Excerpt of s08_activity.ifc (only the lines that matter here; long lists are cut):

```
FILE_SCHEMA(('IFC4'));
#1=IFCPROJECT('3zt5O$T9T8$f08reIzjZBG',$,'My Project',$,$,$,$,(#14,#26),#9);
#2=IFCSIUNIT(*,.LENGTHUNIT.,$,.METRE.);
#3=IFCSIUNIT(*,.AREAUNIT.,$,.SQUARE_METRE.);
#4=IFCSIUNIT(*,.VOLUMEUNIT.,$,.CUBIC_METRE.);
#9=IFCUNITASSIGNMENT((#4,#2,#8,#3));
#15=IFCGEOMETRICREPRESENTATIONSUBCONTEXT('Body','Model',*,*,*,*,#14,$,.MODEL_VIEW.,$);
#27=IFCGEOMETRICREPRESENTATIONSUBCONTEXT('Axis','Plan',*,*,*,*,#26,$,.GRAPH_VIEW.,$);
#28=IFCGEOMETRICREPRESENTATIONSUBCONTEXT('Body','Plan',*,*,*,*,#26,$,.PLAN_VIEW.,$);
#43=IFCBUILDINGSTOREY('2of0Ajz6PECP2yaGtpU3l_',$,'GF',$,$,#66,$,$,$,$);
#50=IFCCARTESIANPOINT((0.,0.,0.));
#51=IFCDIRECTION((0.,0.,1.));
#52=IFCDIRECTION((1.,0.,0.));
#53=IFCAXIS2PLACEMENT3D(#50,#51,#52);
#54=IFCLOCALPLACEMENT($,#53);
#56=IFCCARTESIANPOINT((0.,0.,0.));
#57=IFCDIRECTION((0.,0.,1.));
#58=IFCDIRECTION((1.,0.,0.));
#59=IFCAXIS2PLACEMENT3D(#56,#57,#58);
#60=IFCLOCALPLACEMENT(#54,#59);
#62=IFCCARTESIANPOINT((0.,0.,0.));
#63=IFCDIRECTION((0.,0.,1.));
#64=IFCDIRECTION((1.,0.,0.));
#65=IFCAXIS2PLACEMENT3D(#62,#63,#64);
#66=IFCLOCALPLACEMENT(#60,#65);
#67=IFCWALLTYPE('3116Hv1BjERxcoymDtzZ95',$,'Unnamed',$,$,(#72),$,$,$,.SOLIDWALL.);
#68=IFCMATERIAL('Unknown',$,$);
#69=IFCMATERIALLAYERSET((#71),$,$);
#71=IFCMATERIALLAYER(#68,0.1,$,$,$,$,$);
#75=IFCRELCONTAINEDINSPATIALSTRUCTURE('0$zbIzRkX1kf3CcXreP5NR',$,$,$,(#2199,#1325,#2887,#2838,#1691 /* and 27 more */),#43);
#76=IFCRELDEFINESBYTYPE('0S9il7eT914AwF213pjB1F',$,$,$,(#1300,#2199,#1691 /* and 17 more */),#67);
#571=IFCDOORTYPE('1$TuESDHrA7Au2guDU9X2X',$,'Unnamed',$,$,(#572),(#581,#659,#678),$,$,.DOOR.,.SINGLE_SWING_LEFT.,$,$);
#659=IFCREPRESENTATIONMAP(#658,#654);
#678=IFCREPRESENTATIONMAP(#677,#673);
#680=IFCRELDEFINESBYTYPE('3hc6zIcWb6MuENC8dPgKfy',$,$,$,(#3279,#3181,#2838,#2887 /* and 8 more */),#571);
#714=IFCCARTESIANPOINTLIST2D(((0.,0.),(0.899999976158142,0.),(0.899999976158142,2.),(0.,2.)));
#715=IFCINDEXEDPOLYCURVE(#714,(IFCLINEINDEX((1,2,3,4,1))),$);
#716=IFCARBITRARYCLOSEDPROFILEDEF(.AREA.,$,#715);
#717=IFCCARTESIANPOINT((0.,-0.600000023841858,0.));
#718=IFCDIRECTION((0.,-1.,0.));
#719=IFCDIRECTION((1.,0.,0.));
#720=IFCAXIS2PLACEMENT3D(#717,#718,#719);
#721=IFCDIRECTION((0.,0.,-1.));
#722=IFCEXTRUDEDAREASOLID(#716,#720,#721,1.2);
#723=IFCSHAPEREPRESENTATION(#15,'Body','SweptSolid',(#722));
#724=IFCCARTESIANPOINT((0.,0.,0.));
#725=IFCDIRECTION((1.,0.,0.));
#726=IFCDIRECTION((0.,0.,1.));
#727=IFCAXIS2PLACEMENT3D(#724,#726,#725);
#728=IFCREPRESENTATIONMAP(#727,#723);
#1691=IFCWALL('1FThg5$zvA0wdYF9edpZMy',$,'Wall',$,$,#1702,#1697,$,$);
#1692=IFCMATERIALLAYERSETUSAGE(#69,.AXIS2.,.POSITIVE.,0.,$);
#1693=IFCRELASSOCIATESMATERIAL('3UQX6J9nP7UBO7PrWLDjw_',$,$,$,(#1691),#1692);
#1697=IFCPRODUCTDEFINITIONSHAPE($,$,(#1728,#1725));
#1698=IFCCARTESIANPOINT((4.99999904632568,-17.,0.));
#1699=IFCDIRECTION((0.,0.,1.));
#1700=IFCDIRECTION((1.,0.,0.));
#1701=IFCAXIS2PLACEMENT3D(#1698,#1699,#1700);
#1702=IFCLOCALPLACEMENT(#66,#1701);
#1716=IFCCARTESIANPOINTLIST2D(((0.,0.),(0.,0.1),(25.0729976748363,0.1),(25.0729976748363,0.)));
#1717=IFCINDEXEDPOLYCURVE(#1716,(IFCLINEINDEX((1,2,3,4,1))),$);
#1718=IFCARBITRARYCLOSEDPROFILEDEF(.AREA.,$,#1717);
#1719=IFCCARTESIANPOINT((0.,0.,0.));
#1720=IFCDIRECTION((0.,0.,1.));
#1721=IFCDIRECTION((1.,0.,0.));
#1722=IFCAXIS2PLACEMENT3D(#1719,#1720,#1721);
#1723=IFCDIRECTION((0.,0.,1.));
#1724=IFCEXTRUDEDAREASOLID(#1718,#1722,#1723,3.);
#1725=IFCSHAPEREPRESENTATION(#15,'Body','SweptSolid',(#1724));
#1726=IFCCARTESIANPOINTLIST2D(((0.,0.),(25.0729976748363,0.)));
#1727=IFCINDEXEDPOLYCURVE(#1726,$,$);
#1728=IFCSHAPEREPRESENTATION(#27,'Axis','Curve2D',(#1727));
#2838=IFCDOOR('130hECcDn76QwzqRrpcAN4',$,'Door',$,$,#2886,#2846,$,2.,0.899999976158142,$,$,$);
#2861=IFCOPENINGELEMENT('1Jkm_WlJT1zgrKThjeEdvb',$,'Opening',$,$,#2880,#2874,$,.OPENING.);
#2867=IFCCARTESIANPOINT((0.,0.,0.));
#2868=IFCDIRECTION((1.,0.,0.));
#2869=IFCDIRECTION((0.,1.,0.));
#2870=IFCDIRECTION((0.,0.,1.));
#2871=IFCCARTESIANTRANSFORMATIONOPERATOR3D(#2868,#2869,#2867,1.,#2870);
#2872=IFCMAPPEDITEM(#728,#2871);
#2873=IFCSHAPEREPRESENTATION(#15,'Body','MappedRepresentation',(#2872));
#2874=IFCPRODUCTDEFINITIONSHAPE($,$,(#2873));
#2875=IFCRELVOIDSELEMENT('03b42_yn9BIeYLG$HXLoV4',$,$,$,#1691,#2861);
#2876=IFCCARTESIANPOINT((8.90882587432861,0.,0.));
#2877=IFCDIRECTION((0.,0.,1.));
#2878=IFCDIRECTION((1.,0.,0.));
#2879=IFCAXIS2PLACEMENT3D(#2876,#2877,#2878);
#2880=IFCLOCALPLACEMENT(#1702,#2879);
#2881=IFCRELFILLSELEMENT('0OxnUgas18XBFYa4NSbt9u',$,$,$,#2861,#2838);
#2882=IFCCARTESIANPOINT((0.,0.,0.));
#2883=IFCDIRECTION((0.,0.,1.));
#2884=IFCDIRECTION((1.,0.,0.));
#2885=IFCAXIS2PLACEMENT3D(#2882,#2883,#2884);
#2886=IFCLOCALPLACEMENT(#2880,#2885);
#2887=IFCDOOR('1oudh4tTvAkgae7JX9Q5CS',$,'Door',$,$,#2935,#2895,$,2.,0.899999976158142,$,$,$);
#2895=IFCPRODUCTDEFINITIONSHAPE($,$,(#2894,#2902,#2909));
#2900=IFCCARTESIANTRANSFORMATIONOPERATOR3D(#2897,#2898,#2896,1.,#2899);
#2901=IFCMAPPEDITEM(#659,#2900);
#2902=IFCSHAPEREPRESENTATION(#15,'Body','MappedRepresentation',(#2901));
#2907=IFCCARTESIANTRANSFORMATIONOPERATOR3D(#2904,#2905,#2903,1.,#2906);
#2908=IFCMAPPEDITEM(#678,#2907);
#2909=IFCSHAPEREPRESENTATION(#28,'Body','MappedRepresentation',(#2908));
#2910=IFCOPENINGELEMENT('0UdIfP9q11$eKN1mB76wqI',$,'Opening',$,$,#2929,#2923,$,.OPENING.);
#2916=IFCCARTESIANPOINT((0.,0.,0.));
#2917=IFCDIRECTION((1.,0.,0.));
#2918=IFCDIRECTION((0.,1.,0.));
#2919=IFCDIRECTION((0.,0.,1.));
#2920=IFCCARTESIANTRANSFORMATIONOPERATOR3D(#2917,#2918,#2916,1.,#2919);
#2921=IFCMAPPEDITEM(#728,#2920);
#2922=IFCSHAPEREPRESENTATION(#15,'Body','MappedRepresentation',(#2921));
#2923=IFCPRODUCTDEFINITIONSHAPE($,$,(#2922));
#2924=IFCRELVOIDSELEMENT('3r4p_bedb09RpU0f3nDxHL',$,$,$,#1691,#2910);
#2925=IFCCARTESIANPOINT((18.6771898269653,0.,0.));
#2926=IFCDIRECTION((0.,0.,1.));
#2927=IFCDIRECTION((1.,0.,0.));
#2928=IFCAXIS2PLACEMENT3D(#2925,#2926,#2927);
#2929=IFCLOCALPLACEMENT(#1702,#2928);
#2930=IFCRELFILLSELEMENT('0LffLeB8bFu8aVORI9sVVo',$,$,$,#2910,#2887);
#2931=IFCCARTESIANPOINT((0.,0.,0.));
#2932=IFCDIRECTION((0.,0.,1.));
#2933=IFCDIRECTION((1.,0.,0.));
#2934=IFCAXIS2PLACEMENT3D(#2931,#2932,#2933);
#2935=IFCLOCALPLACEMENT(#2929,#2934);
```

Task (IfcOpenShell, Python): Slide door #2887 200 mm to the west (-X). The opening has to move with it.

```python
import ifcopenshell
import ifcopenshell.api.geometry
import ifcopenshell.util.placement

model = ifcopenshell.open("s08_activity.ifc")

door = model.by_id(2887)
opening = door.FillsVoids[0].RelatingOpeningElement
wall = opening.VoidsElements[0].RelatingBuildingElement

wall_matrix = ifcopenshell.util.placement.get_local_placement(wall.ObjectPlacement)
shift = wall_matrix[:3, 0] * -0.2
before = ifcopenshell.util.placement.get_local_placement(door.ObjectPlacement)[:3, 3].copy()

# The door is placed relative to its opening, so it follows when the opening moves.
matrix = ifcopenshell.util.placement.get_local_placement(opening.ObjectPlacement)
matrix[:3, 3] += shift
ifcopenshell.api.geometry.edit_object_placement(
    model, product=opening, matrix=matrix, is_si=False, should_transform_children=True
)

after = ifcopenshell.util.placement.get_local_placement(door.ObjectPlacement)[:3, 3]
print("door moved by", (after - before).round(3) + 0.0)

model.write("s08_activity_rev.ifc")
```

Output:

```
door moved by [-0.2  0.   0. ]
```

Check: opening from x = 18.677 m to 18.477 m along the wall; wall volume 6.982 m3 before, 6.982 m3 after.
